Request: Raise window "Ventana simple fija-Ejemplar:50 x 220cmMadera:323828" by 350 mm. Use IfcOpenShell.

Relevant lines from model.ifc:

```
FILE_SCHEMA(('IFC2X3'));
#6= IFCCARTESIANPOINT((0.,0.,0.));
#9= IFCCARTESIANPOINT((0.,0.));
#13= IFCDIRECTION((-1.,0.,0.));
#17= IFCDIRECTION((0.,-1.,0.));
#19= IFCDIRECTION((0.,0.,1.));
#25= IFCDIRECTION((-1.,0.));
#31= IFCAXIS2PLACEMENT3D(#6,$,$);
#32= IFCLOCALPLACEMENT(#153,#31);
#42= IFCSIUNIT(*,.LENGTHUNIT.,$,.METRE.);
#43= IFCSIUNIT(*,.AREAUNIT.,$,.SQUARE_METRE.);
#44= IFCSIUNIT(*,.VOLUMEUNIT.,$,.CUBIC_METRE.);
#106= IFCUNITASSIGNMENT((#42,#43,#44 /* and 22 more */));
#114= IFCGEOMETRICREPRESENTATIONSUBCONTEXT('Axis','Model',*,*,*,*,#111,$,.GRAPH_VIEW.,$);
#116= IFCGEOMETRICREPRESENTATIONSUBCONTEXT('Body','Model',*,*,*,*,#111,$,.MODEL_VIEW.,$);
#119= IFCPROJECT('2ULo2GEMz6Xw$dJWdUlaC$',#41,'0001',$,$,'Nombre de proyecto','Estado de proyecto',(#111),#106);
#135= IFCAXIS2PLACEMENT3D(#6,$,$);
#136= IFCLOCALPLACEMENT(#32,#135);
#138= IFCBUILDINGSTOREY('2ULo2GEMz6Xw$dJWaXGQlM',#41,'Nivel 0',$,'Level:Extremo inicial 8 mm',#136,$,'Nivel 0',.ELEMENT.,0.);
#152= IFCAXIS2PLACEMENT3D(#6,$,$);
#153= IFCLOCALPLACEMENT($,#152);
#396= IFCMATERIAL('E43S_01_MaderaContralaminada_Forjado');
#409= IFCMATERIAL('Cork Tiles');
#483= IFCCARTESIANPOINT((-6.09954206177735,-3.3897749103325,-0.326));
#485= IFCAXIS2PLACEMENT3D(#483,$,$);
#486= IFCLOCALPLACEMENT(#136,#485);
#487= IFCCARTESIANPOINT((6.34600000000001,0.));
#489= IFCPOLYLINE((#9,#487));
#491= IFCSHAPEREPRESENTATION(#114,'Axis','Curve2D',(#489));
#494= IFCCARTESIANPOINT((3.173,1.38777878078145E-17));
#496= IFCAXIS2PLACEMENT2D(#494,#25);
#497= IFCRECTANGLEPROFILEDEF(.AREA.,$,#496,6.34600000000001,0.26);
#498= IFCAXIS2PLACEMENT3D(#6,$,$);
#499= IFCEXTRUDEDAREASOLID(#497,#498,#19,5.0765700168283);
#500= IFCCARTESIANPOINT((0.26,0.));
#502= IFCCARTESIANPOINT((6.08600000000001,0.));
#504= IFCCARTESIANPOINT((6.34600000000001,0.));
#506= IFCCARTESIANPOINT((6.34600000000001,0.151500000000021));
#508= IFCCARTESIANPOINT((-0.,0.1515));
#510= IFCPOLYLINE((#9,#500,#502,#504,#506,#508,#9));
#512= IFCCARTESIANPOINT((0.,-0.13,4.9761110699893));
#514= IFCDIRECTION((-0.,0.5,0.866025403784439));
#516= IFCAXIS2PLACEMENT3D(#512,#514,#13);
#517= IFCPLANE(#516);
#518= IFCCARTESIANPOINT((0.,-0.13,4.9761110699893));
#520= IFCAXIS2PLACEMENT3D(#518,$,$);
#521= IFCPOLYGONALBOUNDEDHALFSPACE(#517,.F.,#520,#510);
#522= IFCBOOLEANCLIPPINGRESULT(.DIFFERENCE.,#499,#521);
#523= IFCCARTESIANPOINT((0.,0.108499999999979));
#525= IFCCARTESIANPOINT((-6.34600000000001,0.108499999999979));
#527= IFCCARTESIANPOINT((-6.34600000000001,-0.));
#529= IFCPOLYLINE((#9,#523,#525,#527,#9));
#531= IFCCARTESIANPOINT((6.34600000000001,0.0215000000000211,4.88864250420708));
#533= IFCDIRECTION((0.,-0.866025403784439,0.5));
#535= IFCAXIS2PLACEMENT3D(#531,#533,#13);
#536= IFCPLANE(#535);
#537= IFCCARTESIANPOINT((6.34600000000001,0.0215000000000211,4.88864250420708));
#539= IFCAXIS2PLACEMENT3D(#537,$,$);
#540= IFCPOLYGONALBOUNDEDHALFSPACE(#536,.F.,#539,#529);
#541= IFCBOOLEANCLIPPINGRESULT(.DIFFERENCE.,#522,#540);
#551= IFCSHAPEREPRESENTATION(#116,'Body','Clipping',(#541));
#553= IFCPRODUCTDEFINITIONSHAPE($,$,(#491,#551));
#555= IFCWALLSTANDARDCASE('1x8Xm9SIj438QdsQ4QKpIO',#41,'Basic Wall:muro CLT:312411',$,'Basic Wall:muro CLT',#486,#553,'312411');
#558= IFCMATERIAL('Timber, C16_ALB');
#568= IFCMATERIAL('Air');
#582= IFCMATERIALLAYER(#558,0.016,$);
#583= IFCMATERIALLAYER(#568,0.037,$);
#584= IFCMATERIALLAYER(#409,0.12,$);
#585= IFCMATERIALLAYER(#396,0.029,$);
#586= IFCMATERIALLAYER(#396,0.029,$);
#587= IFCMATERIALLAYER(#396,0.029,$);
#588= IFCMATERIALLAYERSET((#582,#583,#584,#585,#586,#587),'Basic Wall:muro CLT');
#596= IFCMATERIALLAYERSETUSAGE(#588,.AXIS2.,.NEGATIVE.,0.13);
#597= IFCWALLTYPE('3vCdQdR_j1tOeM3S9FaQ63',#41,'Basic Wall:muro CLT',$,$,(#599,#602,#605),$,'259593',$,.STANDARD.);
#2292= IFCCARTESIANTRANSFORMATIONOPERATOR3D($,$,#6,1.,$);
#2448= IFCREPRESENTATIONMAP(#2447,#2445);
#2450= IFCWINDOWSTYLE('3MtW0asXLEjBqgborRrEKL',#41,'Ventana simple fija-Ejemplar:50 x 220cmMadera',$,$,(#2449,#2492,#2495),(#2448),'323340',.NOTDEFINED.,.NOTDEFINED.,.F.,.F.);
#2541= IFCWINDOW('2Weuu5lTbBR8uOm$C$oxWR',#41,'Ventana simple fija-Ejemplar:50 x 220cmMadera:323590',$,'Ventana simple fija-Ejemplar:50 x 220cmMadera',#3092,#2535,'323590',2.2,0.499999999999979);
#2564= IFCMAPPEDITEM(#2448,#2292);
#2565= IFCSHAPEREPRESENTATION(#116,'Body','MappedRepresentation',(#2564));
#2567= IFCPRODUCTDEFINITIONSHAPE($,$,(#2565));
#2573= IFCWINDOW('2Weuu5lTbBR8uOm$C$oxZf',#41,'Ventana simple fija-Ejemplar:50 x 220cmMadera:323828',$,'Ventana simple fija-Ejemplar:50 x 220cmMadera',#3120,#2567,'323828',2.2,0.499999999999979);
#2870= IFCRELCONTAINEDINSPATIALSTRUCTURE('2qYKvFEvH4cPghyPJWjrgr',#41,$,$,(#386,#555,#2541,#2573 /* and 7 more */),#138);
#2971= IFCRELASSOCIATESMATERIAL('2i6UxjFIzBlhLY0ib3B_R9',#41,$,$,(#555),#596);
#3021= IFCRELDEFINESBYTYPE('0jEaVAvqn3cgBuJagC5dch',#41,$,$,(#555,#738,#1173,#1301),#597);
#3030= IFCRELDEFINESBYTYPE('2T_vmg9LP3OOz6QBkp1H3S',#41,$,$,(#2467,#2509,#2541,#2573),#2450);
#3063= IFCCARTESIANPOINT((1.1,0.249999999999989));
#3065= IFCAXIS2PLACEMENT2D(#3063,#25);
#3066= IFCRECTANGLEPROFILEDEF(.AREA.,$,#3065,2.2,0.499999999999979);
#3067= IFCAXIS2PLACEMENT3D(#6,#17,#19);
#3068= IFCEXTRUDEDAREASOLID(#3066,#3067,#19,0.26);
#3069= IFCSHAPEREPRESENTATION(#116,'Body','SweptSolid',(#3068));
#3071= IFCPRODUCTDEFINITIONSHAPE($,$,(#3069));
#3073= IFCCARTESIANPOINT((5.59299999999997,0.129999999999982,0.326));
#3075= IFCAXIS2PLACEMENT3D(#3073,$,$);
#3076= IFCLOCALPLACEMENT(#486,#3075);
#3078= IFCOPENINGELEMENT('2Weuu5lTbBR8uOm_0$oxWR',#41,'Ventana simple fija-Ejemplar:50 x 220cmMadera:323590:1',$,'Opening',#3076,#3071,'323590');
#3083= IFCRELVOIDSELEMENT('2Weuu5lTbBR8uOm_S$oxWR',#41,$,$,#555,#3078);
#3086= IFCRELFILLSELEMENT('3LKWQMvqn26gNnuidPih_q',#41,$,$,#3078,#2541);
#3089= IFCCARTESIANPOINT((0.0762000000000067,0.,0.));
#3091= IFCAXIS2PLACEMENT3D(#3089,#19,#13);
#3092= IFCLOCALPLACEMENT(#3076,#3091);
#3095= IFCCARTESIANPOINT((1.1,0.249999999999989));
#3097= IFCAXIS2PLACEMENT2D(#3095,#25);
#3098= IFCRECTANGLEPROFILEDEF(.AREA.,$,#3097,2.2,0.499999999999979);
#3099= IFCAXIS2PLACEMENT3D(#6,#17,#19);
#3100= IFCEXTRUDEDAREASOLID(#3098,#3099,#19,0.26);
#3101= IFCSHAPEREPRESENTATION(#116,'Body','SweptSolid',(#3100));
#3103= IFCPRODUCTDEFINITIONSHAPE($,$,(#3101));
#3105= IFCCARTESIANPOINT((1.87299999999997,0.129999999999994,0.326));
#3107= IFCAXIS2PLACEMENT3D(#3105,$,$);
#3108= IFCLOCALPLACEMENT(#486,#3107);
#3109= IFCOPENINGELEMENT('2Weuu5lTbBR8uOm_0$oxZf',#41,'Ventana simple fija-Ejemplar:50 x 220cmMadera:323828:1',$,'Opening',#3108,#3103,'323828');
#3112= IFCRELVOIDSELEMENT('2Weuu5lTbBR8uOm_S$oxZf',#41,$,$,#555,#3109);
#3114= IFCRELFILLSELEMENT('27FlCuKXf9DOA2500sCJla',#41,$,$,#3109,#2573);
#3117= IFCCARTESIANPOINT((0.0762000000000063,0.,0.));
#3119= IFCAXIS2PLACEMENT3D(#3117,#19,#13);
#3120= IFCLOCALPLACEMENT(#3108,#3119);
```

```python
import numpy as np
import ifcopenshell
import ifcopenshell.api.geometry
import ifcopenshell.util.placement
import ifcopenshell.util.unit

model = ifcopenshell.open("model.ifc")
unit_scale = ifcopenshell.util.unit.calculate_unit_scale(model)

window = model.by_guid("2Weuu5lTbBR8uOm$C$oxZf")
opening = window.FillsVoids[0].RelatingOpeningElement
dz = 0.35 / unit_scale

shift = np.array([0.0, 0.0, dz])
# The window is placed relative to its opening, so it follows when the opening moves.
matrix = ifcopenshell.util.placement.get_local_placement(opening.ObjectPlacement)
matrix[:3, 3] += shift
ifcopenshell.api.geometry.edit_object_placement(
    model, product=opening, matrix=matrix, is_si=False, should_transform_children=True
)

print(f"moved by {dz * unit_scale:+.3f} m")

model.write("model_updated.ifc")
```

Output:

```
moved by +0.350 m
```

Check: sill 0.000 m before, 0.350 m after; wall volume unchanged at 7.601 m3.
